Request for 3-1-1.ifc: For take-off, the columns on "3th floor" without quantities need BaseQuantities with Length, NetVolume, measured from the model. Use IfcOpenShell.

First a look at what the model holds.

```python
import ifcopenshell
import ifcopenshell.util.element
import ifcopenshell.util.unit

model = ifcopenshell.open("3-1-1.ifc")
print(model.schema)
for unit_type in ("LENGTHUNIT", "AREAUNIT", "VOLUMEUNIT"):
    print(unit_type, ifcopenshell.util.unit.calculate_unit_scale(model, unit_type))
storey = next(s for s in model.by_type("IfcBuildingStorey") if s.Name == "3th floor")
columns = [e for e in ifcopenshell.util.element.get_decomposition(storey) if e.is_a("IfcColumn")]
for e in sorted(columns, key=lambda e: e.id()):
    print(e.id(), e.is_a(), e.Name, list(ifcopenshell.util.element.get_psets(e, qtos_only=True)), sep=" | ")
```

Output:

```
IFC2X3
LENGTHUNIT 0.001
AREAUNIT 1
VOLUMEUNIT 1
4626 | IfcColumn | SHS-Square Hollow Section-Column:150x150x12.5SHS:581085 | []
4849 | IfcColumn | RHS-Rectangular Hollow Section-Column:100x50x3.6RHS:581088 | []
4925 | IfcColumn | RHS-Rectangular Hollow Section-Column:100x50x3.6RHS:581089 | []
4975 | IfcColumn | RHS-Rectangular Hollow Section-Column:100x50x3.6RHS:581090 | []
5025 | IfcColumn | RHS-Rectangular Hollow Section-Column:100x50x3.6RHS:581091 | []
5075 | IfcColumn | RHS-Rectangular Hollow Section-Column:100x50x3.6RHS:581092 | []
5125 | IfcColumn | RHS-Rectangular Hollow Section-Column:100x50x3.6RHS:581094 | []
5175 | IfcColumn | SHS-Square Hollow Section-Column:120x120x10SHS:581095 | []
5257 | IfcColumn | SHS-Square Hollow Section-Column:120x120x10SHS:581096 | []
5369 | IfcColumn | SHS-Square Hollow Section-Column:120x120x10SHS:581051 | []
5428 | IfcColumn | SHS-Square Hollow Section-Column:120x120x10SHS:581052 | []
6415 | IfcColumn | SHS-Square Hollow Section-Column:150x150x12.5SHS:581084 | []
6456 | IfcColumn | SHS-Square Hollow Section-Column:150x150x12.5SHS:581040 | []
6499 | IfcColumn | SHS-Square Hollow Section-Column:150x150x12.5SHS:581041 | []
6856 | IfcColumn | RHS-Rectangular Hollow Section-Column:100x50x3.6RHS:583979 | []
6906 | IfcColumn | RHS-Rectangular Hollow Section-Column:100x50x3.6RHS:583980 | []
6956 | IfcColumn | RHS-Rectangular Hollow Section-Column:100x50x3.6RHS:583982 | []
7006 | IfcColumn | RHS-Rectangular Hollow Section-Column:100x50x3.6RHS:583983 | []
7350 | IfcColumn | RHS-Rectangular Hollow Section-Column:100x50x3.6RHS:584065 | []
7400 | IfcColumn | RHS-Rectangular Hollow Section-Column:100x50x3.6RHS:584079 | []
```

```python
import ifcopenshell
import ifcopenshell.api.pset
import ifcopenshell.geom
import ifcopenshell.util.element
import ifcopenshell.util.shape
import ifcopenshell.util.unit

model = ifcopenshell.open("3-1-1.ifc")
unit_scale = ifcopenshell.util.unit.calculate_unit_scale(model)
volume_scale = ifcopenshell.util.unit.calculate_unit_scale(model, "VOLUMEUNIT")
settings = ifcopenshell.geom.settings()

storey = next(s for s in model.by_type("IfcBuildingStorey") if s.Name == "3th floor")
columns = [e for e in ifcopenshell.util.element.get_decomposition(storey) if e.is_a("IfcColumn")]

for e in sorted(columns, key=lambda e: e.id()):
    if ifcopenshell.util.element.get_psets(e, qtos_only=True, should_inherit=False):
        continue
    # Geometry comes back in metres, in the element's own axes.
    shape = ifcopenshell.geom.create_shape(settings, e)
    values = {
        "Length": ifcopenshell.util.shape.get_z(shape.geometry) / unit_scale,
        "NetVolume": ifcopenshell.util.shape.get_volume(shape.geometry) / volume_scale,
    }
    qto = ifcopenshell.api.pset.add_qto(model, product=e, name="BaseQuantities")
    ifcopenshell.api.pset.edit_qto(model, qto=qto, properties=values)
    print(e.id(), {k: round(v, 3) for k, v in values.items()})

model.write("3-1-1_edited.ifc")
```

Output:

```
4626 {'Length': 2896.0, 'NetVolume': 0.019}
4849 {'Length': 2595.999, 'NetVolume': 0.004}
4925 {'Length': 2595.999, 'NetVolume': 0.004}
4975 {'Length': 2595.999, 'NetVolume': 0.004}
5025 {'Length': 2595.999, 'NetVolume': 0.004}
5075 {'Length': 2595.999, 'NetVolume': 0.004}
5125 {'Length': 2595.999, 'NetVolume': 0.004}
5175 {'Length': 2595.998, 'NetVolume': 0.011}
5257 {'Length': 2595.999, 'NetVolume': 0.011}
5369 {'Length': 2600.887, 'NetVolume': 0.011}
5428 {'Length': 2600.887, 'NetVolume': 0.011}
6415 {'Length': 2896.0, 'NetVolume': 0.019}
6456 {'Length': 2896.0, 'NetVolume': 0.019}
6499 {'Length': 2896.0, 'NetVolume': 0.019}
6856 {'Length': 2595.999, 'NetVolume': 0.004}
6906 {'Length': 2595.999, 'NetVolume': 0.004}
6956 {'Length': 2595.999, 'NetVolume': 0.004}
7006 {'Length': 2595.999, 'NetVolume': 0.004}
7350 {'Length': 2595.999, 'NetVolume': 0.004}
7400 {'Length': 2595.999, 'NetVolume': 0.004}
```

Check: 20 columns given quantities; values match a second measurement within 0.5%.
